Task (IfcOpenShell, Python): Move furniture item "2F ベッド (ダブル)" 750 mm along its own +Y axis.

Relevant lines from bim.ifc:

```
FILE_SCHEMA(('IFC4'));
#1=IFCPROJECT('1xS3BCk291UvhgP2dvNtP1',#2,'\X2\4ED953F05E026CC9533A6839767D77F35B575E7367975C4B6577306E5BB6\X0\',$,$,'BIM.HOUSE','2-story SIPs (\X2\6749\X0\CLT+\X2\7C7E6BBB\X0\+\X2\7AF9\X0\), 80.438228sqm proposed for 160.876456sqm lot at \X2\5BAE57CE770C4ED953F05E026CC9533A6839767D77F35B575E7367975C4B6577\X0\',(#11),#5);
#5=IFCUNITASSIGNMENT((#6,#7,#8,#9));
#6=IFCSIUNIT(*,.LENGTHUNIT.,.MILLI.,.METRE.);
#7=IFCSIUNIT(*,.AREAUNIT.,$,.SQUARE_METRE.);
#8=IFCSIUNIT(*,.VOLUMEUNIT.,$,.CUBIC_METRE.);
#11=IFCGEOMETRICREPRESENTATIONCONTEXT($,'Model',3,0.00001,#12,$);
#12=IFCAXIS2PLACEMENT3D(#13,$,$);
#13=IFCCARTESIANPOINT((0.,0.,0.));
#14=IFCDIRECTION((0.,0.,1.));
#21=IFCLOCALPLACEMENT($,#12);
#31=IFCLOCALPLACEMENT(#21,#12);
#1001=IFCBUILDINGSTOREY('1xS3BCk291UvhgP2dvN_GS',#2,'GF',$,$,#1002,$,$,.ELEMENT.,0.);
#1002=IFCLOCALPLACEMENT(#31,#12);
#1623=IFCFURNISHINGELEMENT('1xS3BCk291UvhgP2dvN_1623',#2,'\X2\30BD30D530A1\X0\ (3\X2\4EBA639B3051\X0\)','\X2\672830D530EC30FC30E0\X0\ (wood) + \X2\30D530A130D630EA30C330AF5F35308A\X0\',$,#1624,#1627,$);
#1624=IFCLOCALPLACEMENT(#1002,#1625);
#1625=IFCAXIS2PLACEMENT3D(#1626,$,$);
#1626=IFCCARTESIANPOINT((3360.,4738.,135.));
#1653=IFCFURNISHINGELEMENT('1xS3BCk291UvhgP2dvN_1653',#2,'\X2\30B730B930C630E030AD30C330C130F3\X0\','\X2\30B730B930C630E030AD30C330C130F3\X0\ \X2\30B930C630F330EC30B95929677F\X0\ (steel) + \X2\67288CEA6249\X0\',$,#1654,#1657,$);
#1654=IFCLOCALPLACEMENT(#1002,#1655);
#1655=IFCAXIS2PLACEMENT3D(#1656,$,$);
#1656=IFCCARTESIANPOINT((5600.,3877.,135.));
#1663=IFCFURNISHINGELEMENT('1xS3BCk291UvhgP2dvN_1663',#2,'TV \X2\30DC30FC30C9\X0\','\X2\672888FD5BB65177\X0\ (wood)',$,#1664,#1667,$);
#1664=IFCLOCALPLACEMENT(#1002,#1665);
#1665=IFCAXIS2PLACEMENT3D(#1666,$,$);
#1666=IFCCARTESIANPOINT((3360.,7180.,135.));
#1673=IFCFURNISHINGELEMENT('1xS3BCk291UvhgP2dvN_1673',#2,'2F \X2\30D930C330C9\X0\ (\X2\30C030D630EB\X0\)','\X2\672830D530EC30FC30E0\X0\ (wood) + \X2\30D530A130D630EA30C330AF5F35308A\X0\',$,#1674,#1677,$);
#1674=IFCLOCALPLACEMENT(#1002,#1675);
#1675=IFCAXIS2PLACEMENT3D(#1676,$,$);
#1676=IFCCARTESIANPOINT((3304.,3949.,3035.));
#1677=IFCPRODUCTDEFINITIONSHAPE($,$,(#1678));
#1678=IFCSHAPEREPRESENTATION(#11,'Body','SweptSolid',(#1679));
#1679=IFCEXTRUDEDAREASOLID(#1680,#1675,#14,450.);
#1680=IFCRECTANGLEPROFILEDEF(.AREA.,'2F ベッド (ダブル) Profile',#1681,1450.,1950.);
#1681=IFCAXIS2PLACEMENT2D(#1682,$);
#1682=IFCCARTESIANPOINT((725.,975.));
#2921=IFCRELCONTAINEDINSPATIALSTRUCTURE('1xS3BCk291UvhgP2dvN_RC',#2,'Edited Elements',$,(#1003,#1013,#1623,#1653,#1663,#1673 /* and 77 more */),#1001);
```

```python
import ifcopenshell
import ifcopenshell.api.geometry
import ifcopenshell.util.placement

model = ifcopenshell.open("bim.ifc")

item = model.by_guid("1xS3BCk291UvhgP2dvN_1673")
matrix = ifcopenshell.util.placement.get_local_placement(item.ObjectPlacement)
matrix[:3, 3] += matrix[:3, 1] * 750.0
ifcopenshell.api.geometry.edit_object_placement(model, product=item, matrix=matrix, is_si=False)

print(ifcopenshell.util.placement.get_local_placement(item.ObjectPlacement).round(3) + 0.0)

model.write("bim-out.ifc")
```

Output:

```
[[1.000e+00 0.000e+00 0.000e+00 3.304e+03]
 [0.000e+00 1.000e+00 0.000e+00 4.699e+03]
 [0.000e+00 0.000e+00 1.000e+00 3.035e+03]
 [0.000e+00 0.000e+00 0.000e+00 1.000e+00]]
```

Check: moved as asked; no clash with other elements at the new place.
